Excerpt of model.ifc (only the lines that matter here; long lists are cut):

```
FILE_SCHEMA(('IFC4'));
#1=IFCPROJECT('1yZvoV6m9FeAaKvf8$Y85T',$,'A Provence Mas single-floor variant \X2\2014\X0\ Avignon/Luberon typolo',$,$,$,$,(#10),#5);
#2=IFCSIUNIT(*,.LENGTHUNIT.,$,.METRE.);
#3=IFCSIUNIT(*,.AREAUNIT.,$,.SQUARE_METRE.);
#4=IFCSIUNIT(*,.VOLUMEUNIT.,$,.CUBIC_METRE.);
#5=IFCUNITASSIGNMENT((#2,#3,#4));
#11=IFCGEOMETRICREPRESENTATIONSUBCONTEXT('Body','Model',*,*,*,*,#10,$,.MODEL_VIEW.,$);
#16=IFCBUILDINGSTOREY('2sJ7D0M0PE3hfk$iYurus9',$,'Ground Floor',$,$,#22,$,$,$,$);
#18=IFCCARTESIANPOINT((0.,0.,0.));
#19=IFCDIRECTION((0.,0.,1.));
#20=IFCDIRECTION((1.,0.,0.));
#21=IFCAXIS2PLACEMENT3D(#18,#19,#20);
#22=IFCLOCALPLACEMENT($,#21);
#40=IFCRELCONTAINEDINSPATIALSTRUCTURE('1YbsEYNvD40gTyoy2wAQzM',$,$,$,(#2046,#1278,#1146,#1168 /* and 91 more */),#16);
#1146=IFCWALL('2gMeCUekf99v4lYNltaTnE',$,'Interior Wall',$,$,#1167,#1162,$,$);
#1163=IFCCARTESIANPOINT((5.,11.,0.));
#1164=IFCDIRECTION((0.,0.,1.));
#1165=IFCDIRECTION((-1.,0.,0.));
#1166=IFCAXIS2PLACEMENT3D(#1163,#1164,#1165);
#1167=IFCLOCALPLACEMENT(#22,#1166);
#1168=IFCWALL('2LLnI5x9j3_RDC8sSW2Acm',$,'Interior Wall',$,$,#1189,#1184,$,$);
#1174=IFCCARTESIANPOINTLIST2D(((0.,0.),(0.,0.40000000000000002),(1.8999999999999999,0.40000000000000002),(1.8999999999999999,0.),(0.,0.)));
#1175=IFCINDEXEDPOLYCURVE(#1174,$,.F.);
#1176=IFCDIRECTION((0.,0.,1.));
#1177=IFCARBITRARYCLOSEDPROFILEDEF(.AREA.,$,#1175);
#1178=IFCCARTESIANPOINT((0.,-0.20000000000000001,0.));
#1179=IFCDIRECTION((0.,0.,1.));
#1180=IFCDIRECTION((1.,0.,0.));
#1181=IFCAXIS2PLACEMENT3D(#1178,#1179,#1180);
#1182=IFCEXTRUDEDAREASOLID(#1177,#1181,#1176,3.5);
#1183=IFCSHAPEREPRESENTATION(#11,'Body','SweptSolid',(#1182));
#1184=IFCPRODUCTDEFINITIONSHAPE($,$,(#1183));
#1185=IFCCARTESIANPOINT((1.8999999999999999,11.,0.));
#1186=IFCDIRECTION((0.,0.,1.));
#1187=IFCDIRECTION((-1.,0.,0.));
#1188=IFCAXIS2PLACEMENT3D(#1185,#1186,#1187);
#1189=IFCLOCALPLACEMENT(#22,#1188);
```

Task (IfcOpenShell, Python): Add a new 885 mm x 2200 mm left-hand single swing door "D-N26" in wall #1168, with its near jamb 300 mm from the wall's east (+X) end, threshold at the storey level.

```python
import numpy as np
import ifcopenshell
import ifcopenshell.api.feature
import ifcopenshell.api.geometry
import ifcopenshell.api.root
import ifcopenshell.api.spatial
import ifcopenshell.geom
import ifcopenshell.util.element
import ifcopenshell.util.placement
import ifcopenshell.util.representation
import ifcopenshell.util.shape
import ifcopenshell.util.unit

model = ifcopenshell.open("model.ifc")
unit_scale = ifcopenshell.util.unit.calculate_unit_scale(model)
settings = ifcopenshell.geom.settings()


def volume(element):
    """Net volume in cubic metres, openings subtracted."""
    shape = ifcopenshell.geom.create_shape(settings, element)
    return ifcopenshell.util.shape.get_volume(shape.geometry)


wall = model.by_id(1168)
storey = ifcopenshell.util.element.get_container(wall, ifc_class="IfcBuildingStorey")
context = ifcopenshell.util.representation.get_context(model, "Model", "Body", "MODEL_VIEW")
before = volume(wall)

width, height, from_end, sill = 0.885, 2.2, 0.3, 0.0  # metres

# The wall runs along its own X axis, and the end named is its -X end.
wall_shape = ifcopenshell.geom.create_shape(settings, wall)
x, y, z = ifcopenshell.util.shape.get_vertices(wall_shape.geometry).T
start = x.min() + from_end
face, thickness = float(y.min()), float(y.max() - y.min())
wall_matrix = ifcopenshell.util.placement.get_local_placement(wall.ObjectPlacement)
level = ifcopenshell.util.placement.get_local_placement(storey.ObjectPlacement)[2, 3]


def in_wall(x, y):
    """Placement at x, y metres in the wall's axes, at sill height."""
    matrix = wall_matrix.copy()
    matrix[:, 3] = wall_matrix @ np.array([x / unit_scale, y / unit_scale, 0.0, 1.0])
    matrix[2, 3] = level + sill / unit_scale
    return matrix


# Opening: a box that overshoots both wall faces by 50 mm.
opening = ifcopenshell.api.root.create_entity(model, ifc_class="IfcOpeningElement", predefined_type="OPENING")
box = ifcopenshell.api.geometry.add_wall_representation(
    model, context=context, length=width, height=height, thickness=thickness + 0.1
)
ifcopenshell.api.geometry.assign_representation(model, product=opening, representation=box)
ifcopenshell.api.geometry.edit_object_placement(model, product=opening, matrix=in_wall(start, face - 0.05), is_si=False)
ifcopenshell.api.feature.add_feature(model, feature=opening, element=wall)

door = ifcopenshell.api.root.create_entity(model, ifc_class="IfcDoor", name="D-N26", predefined_type="DOOR")
door.OverallWidth, door.OverallHeight = width / unit_scale, height / unit_scale
door.OperationType = "SINGLE_SWING_LEFT"
body = ifcopenshell.api.geometry.add_door_representation(
    model,
    context=context,
    overall_width=door.OverallWidth,
    overall_height=door.OverallHeight,
    operation_type="SINGLE_SWING_LEFT",
    lining_properties={"LiningDepth": thickness / unit_scale, "ThresholdDepth": thickness / unit_scale},
)
ifcopenshell.api.geometry.assign_representation(model, product=door, representation=body)
ifcopenshell.api.spatial.assign_container(model, products=[door], relating_structure=storey)
ifcopenshell.api.feature.add_filling(model, opening=opening, element=door)

# The lining spans the wall, so the door starts at the wall face.
ifcopenshell.api.geometry.edit_object_placement(model, product=door, matrix=in_wall(start, face), is_si=False)

after = volume(wall)

print(f"wall volume {before:.3f} -> {after:.3f} m3")

model.write("model_edited.ifc")
```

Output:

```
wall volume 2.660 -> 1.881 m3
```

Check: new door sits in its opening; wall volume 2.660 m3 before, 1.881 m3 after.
